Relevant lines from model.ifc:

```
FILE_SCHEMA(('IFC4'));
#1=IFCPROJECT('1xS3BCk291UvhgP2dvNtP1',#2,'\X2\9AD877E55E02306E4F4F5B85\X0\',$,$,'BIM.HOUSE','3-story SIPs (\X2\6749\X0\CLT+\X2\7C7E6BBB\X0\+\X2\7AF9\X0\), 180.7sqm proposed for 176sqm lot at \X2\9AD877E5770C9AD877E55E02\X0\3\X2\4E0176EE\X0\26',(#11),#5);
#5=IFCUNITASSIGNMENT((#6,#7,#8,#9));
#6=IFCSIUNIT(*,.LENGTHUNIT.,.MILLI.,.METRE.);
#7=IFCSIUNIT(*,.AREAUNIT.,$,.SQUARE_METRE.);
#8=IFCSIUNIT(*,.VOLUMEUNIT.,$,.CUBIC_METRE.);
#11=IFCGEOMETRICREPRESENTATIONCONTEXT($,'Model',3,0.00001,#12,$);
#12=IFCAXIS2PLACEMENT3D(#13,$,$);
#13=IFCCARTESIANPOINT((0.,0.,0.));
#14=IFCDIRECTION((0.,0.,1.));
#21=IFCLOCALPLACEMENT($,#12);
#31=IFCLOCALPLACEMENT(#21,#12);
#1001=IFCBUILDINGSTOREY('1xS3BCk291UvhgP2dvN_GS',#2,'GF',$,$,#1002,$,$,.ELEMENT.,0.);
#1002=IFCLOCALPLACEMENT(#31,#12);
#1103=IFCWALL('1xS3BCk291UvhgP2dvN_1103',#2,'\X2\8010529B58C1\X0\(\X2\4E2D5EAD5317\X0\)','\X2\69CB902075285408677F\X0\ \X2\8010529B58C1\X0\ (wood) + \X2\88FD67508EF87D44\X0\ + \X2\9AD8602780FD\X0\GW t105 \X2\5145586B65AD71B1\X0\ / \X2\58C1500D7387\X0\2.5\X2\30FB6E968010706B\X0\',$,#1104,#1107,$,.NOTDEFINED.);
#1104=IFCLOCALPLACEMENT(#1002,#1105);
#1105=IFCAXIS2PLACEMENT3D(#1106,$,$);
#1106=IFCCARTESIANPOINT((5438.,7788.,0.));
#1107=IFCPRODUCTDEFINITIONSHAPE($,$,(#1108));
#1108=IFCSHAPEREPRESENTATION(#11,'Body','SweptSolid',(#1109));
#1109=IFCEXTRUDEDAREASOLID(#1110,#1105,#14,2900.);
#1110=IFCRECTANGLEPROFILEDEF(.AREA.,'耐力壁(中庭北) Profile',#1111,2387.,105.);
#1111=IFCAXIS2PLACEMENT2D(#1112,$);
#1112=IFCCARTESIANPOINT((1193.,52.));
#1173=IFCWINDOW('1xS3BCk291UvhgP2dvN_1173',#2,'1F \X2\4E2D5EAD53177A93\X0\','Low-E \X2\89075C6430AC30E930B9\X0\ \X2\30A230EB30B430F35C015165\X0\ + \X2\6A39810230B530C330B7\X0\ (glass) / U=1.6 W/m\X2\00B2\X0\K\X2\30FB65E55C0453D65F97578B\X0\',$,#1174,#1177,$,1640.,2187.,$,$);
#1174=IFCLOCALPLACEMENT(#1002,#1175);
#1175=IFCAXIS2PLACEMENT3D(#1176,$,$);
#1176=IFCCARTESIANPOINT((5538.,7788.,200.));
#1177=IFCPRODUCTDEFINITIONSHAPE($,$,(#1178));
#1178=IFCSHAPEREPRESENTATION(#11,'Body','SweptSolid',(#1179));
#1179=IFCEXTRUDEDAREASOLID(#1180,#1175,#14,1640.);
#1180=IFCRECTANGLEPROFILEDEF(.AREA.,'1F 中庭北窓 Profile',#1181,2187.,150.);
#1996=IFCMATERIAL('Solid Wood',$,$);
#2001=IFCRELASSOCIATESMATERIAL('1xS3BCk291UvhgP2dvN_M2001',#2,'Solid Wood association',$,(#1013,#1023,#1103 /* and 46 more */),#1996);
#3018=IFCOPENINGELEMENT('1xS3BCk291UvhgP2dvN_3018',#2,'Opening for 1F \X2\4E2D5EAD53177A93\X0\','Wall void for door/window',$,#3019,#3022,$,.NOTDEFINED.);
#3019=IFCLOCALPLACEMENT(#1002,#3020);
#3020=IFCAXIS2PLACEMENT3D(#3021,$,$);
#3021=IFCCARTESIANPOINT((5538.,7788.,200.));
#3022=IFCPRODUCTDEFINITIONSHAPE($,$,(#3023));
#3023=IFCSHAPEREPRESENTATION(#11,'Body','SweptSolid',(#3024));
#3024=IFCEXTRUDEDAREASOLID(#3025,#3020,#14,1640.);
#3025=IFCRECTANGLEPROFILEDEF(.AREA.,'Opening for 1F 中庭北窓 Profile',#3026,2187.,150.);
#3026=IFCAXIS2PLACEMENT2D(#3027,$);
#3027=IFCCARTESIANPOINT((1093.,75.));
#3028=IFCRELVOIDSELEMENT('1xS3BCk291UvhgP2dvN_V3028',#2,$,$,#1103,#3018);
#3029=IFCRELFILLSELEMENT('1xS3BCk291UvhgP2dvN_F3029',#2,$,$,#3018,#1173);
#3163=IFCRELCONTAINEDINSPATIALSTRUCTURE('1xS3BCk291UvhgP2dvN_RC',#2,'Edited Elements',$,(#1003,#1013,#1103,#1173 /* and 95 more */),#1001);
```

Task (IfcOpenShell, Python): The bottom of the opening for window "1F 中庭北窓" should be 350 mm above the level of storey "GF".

```python
import numpy as np
import ifcopenshell
import ifcopenshell.api.geometry
import ifcopenshell.geom
import ifcopenshell.util.element
import ifcopenshell.util.placement
import ifcopenshell.util.shape
import ifcopenshell.util.unit

model = ifcopenshell.open("model.ifc")
unit_scale = ifcopenshell.util.unit.calculate_unit_scale(model)

window = model.by_guid("1xS3BCk291UvhgP2dvN_1173")
opening = window.FillsVoids[0].RelatingOpeningElement
storey = ifcopenshell.util.element.get_container(window, ifc_class="IfcBuildingStorey")
level = ifcopenshell.util.placement.get_local_placement(storey.ObjectPlacement)[2, 3]

# The opening's origin need not be at the sill, so measure its lowest point.
shape = ifcopenshell.geom.create_shape(ifcopenshell.geom.settings(), opening)
bottom = ifcopenshell.util.shape.get_shape_bottom_elevation(shape, shape.geometry) / unit_scale
dz = level + 0.35 / unit_scale - bottom

shift = np.array([0.0, 0.0, dz])
# The window is not placed relative to its opening, so move both.
for product in (opening, window):
    matrix = ifcopenshell.util.placement.get_local_placement(product.ObjectPlacement)
    matrix[:3, 3] += shift
    ifcopenshell.api.geometry.edit_object_placement(model, product=product, matrix=matrix, is_si=False)

print(f"moved by {dz * unit_scale:+.3f} m")

model.write("model_v2.ifc")
```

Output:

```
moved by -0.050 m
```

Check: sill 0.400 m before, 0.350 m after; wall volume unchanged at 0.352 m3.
